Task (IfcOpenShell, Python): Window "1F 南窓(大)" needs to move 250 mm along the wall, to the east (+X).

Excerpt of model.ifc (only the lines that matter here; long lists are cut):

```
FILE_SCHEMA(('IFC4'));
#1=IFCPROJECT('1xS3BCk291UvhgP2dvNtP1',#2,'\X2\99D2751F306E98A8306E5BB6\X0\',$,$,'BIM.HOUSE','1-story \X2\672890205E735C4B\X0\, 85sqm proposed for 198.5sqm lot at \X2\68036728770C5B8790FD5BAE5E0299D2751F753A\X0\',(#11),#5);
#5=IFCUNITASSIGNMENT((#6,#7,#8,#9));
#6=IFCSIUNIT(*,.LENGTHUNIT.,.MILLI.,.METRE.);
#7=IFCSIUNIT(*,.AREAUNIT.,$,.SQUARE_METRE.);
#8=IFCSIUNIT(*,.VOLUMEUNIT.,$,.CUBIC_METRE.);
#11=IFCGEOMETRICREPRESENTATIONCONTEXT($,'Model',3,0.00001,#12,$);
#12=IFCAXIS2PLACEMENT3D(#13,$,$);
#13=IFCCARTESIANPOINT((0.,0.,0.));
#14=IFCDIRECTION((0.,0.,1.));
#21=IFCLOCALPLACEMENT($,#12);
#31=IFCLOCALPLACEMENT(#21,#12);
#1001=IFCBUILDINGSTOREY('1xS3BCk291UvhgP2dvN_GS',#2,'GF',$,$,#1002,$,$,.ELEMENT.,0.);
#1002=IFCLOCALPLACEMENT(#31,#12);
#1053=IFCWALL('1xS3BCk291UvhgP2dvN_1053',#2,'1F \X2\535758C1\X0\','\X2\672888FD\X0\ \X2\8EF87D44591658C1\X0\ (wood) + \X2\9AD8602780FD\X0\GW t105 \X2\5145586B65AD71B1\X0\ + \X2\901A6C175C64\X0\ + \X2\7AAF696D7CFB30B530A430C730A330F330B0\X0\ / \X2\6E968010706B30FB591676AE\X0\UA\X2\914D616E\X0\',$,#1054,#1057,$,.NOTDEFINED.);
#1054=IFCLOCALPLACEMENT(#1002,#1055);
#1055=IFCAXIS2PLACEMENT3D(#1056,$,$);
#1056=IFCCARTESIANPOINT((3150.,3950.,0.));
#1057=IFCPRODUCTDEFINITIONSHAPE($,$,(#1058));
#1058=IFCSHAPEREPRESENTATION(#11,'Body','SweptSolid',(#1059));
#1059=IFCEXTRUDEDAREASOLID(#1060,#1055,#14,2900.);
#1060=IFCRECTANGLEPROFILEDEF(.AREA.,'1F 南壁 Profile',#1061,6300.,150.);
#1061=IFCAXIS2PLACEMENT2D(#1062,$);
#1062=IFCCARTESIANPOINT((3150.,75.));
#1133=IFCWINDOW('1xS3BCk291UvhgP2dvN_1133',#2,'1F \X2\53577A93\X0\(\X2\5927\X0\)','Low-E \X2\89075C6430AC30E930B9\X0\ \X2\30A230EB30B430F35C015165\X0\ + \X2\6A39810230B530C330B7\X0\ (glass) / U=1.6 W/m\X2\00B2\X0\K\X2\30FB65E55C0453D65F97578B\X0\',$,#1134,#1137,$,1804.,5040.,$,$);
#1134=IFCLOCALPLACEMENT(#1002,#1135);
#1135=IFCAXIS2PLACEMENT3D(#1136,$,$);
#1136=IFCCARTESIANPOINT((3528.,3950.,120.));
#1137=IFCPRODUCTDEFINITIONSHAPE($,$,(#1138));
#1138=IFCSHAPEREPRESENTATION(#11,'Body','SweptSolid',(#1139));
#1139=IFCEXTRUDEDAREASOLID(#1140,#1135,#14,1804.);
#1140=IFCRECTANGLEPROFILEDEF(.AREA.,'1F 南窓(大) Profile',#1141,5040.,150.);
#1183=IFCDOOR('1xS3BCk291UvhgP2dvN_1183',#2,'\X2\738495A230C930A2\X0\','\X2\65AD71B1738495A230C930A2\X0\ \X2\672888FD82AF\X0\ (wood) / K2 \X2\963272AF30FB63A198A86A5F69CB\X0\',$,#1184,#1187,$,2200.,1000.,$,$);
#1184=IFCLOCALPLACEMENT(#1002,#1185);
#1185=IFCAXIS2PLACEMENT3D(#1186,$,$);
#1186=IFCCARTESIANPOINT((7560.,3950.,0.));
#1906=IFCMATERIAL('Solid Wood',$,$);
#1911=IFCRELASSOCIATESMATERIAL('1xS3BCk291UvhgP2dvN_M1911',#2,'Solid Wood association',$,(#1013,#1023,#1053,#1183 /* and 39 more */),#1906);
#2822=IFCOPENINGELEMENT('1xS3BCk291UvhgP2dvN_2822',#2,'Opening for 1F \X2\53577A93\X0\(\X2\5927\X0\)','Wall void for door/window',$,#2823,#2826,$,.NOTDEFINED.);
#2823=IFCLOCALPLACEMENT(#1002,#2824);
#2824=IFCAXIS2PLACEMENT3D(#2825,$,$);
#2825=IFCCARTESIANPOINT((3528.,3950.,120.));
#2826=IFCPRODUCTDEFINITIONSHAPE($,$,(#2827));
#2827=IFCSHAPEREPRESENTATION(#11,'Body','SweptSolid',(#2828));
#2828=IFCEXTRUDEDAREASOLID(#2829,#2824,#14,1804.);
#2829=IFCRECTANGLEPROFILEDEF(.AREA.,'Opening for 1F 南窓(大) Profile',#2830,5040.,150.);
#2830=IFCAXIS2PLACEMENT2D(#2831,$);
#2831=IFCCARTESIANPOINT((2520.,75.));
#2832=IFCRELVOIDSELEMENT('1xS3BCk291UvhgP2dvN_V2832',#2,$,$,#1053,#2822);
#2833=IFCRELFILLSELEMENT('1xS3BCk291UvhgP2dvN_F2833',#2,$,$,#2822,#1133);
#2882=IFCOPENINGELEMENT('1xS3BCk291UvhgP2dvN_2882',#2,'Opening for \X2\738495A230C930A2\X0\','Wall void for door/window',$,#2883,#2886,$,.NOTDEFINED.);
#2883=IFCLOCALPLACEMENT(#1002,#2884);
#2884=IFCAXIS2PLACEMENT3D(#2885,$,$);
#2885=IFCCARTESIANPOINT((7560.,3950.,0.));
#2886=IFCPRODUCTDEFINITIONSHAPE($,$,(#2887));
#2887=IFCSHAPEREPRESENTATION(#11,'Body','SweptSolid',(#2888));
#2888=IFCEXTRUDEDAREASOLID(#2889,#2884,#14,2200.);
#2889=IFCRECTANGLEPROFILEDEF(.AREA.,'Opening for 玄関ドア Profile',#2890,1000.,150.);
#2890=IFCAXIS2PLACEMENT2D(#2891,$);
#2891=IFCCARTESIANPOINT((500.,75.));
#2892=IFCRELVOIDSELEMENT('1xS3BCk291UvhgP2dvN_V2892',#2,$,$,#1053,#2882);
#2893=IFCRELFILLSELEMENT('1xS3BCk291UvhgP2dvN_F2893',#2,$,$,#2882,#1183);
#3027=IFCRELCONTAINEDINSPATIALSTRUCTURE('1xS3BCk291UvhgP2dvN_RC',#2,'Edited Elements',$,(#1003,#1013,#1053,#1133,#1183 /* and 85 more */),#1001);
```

```python
import ifcopenshell
import ifcopenshell.api.geometry
import ifcopenshell.util.placement

model = ifcopenshell.open("model.ifc")

window = model.by_guid("1xS3BCk291UvhgP2dvN_1133")
opening = window.FillsVoids[0].RelatingOpeningElement
wall = opening.VoidsElements[0].RelatingBuildingElement

wall_matrix = ifcopenshell.util.placement.get_local_placement(wall.ObjectPlacement)
shift = wall_matrix[:3, 0] * 250.0
before = ifcopenshell.util.placement.get_local_placement(window.ObjectPlacement)[:3, 3].copy()

# The window is not placed relative to its opening, so move both.
for product in (opening, window):
    matrix = ifcopenshell.util.placement.get_local_placement(product.ObjectPlacement)
    matrix[:3, 3] += shift
    ifcopenshell.api.geometry.edit_object_placement(model, product=product, matrix=matrix, is_si=False)

after = ifcopenshell.util.placement.get_local_placement(window.ObjectPlacement)[:3, 3]
print("window moved by", (after - before).round(3) + 0.0)

model.write("model_rev.ifc")
```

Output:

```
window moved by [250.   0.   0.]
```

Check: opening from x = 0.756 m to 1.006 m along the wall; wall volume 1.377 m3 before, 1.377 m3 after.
